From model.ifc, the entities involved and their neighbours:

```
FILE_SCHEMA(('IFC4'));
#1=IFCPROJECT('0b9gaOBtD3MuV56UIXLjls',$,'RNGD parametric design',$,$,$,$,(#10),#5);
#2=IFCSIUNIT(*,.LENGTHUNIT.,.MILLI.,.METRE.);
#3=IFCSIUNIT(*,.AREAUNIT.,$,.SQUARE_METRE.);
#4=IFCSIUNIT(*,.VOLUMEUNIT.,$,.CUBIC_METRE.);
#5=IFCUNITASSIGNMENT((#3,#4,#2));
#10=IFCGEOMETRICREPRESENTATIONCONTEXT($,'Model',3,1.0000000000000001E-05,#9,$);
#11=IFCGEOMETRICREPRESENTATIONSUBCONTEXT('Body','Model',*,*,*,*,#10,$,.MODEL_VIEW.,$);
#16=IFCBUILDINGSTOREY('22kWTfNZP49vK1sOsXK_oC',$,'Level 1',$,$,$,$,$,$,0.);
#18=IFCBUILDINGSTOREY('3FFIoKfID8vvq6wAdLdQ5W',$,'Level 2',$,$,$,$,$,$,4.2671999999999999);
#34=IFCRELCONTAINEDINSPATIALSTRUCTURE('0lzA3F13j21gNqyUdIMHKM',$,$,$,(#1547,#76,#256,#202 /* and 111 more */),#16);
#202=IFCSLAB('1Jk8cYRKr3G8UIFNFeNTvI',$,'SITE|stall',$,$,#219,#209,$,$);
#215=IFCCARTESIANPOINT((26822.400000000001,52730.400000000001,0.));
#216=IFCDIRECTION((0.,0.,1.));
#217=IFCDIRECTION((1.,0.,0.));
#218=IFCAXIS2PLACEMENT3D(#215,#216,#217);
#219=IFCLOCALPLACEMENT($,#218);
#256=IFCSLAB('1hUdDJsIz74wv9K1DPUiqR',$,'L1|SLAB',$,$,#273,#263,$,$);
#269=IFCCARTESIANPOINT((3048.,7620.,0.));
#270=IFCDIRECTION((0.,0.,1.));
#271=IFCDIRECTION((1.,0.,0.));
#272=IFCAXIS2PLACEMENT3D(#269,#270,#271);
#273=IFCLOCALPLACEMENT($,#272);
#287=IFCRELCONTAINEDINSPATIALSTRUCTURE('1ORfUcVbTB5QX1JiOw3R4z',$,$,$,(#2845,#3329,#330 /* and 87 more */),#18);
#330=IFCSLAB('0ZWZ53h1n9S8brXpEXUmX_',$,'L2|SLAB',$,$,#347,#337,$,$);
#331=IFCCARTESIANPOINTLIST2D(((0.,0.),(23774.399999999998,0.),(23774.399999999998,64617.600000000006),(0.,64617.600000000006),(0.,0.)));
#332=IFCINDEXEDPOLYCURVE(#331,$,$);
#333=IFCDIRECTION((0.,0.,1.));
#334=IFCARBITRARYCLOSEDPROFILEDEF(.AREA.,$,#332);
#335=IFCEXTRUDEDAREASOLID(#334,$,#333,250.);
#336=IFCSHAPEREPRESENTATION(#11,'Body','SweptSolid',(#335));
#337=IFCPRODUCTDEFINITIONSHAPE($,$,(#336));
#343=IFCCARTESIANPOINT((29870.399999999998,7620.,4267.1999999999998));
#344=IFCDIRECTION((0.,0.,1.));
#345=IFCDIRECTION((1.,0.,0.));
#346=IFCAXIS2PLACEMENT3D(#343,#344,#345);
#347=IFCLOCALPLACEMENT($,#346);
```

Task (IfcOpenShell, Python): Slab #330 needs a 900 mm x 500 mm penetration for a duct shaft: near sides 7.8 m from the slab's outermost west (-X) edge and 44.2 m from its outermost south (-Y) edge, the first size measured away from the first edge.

```python
import numpy as np
import ifcopenshell
import ifcopenshell.api.feature
import ifcopenshell.api.geometry
import ifcopenshell.api.root
import ifcopenshell.geom
import ifcopenshell.util.placement
import ifcopenshell.util.representation
import ifcopenshell.util.shape
import ifcopenshell.util.unit

model = ifcopenshell.open("model.ifc")
unit_scale = ifcopenshell.util.unit.calculate_unit_scale(model)
settings = ifcopenshell.geom.settings()


def volume(element):
    """Net volume in cubic metres, openings subtracted."""
    shape = ifcopenshell.geom.create_shape(settings, element)
    return ifcopenshell.util.shape.get_volume(shape.geometry)


slab = model.by_guid("0ZWZ53h1n9S8brXpEXUmX_")
before = volume(slab)

# Extent in the slab's own axes, in metres. The edges named are its -X and -Y sides.
slab_shape = ifcopenshell.geom.create_shape(settings, slab)
vertices = ifcopenshell.util.shape.get_vertices(slab_shape.geometry)
x_min, y_min, bottom = vertices.min(axis=0)
top = vertices[:, 2].max()

opening = ifcopenshell.api.root.create_entity(model, ifc_class="IfcOpeningElement", name="Duct shaft opening", predefined_type="OPENING")
context = ifcopenshell.util.representation.get_context(model, "Model", "Body", "MODEL_VIEW")
width, depth = 0.9, 0.5
outline = [(0.0, 0.0), (width, 0.0), (width, depth), (0.0, depth), (0.0, 0.0)]
# Overshoot both faces by 50 mm so the cut is clean.
shape = ifcopenshell.api.geometry.add_slab_representation(
    model, context=context, depth=top - bottom + 0.1, polyline=outline
)
ifcopenshell.api.geometry.assign_representation(model, product=opening, representation=shape)

matrix = ifcopenshell.util.placement.get_local_placement(slab.ObjectPlacement)
matrix[:, 3] = matrix @ np.append(np.array([x_min + 7.8, y_min + 44.2, bottom - 0.05]) / unit_scale, 1.0)
ifcopenshell.api.geometry.edit_object_placement(model, product=opening, matrix=matrix, is_si=False)
ifcopenshell.api.feature.add_feature(model, feature=opening, element=slab)

after = volume(slab)

print(f"slab volume {before:.3f} -> {after:.3f} m3")

model.write("model_v2.ifc")
```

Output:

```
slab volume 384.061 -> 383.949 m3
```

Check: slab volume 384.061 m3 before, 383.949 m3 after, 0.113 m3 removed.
